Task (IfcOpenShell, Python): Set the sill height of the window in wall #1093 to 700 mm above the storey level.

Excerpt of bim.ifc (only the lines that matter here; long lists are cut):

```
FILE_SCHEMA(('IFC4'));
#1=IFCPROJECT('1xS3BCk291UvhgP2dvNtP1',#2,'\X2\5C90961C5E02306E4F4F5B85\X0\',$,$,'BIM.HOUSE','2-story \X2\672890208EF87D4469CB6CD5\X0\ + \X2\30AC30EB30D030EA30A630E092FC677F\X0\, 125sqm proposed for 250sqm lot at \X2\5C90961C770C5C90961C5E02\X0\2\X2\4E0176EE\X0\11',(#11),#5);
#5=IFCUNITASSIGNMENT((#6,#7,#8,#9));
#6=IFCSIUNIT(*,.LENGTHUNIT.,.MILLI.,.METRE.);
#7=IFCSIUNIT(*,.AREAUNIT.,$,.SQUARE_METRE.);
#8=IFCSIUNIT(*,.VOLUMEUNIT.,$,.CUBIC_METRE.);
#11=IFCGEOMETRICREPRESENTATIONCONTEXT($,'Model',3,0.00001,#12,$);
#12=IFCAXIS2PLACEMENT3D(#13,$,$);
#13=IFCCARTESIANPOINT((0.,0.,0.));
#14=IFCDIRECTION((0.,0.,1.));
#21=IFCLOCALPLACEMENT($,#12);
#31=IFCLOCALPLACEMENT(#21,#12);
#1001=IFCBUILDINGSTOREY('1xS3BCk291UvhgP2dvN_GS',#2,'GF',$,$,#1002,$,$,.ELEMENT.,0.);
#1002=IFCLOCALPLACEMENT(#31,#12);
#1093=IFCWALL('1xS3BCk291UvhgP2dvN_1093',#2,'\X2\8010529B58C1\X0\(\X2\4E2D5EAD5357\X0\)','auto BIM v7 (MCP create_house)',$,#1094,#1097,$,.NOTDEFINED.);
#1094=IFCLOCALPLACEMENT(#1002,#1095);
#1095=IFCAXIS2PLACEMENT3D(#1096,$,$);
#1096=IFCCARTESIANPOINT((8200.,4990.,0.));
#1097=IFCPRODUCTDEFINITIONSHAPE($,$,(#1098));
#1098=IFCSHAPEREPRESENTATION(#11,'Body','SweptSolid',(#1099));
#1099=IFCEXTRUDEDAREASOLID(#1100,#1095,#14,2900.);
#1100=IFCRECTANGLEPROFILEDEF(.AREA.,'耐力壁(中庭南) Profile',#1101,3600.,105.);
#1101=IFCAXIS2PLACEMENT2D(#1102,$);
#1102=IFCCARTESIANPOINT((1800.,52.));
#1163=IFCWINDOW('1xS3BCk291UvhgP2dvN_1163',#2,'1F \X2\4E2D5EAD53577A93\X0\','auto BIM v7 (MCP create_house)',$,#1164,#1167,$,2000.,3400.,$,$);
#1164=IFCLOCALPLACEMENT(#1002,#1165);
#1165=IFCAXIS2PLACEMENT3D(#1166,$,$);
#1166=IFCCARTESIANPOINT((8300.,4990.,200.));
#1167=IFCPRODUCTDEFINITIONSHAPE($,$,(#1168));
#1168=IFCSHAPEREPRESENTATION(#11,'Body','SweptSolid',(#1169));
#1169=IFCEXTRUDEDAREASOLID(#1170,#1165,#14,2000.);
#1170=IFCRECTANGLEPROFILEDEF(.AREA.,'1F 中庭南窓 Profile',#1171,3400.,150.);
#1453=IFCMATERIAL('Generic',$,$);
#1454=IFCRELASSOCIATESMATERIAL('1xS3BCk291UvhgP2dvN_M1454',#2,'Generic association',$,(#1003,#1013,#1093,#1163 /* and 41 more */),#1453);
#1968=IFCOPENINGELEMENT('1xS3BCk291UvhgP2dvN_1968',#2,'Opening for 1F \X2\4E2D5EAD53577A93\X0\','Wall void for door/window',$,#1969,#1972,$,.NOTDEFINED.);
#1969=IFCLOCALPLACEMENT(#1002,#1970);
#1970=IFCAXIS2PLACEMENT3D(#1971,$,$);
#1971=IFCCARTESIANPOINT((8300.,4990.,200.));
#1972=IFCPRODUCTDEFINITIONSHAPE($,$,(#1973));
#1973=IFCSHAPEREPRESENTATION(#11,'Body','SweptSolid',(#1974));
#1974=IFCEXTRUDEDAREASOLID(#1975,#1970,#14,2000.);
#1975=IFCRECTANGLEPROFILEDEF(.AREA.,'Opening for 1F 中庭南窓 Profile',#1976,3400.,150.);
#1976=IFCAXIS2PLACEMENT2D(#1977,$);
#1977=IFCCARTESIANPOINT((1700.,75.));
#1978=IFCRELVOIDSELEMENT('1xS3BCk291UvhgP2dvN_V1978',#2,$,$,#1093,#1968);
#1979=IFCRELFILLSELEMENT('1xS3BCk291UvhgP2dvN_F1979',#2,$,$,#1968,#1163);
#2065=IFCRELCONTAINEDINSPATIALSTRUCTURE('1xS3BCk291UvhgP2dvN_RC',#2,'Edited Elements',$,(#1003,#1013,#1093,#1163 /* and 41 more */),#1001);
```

```python
import numpy as np
import ifcopenshell
import ifcopenshell.api.geometry
import ifcopenshell.geom
import ifcopenshell.util.element
import ifcopenshell.util.placement
import ifcopenshell.util.shape
import ifcopenshell.util.unit

model = ifcopenshell.open("bim.ifc")
unit_scale = ifcopenshell.util.unit.calculate_unit_scale(model)

window = model.by_guid("1xS3BCk291UvhgP2dvN_1163")
opening = window.FillsVoids[0].RelatingOpeningElement
storey = ifcopenshell.util.element.get_container(window, ifc_class="IfcBuildingStorey")
level = ifcopenshell.util.placement.get_local_placement(storey.ObjectPlacement)[2, 3]

# The opening's origin need not be at the sill, so measure its lowest point.
shape = ifcopenshell.geom.create_shape(ifcopenshell.geom.settings(), opening)
bottom = ifcopenshell.util.shape.get_shape_bottom_elevation(shape, shape.geometry) / unit_scale
dz = level + 0.7 / unit_scale - bottom

shift = np.array([0.0, 0.0, dz])
# The window is not placed relative to its opening, so move both.
for product in (opening, window):
    matrix = ifcopenshell.util.placement.get_local_placement(product.ObjectPlacement)
    matrix[:3, 3] += shift
    ifcopenshell.api.geometry.edit_object_placement(model, product=product, matrix=matrix, is_si=False)

print(f"moved by {dz * unit_scale:+.3f} m")

model.write("bim_updated.ifc")
```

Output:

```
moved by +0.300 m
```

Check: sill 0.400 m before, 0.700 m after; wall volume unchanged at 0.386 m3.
